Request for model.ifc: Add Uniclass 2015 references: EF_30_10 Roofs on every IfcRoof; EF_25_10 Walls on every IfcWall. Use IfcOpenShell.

First a look at what the model holds.

```python
import ifcopenshell

model = ifcopenshell.open("model.ifc")
print(model.schema)
print("classifications:", [c.Name for c in model.by_type("IfcClassification")])
for ifc_class in ("IfcDoor", "IfcRoof", "IfcStair", "IfcWall", "IfcWindow"):
    print(ifc_class, len(model.by_type(ifc_class)))
```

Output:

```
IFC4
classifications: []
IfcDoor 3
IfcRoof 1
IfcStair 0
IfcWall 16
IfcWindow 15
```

```python
import ifcopenshell
import ifcopenshell.api.classification

model = ifcopenshell.open("model.ifc")

system = ifcopenshell.api.classification.add_classification(model, classification="Uniclass 2015")

codes = {
    "IfcRoof": ("EF_30_10", "Roofs"),
    "IfcWall": ("EF_25_10", "Walls"),
}
for ifc_class, (code, name) in codes.items():
    products = model.by_type(ifc_class)
    ifcopenshell.api.classification.add_reference(
        model, products=products, classification=system, identification=code, name=name
    )
    print(code, len(products))

model.write("model_v2.ifc")
```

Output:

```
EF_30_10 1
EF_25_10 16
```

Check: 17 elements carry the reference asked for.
